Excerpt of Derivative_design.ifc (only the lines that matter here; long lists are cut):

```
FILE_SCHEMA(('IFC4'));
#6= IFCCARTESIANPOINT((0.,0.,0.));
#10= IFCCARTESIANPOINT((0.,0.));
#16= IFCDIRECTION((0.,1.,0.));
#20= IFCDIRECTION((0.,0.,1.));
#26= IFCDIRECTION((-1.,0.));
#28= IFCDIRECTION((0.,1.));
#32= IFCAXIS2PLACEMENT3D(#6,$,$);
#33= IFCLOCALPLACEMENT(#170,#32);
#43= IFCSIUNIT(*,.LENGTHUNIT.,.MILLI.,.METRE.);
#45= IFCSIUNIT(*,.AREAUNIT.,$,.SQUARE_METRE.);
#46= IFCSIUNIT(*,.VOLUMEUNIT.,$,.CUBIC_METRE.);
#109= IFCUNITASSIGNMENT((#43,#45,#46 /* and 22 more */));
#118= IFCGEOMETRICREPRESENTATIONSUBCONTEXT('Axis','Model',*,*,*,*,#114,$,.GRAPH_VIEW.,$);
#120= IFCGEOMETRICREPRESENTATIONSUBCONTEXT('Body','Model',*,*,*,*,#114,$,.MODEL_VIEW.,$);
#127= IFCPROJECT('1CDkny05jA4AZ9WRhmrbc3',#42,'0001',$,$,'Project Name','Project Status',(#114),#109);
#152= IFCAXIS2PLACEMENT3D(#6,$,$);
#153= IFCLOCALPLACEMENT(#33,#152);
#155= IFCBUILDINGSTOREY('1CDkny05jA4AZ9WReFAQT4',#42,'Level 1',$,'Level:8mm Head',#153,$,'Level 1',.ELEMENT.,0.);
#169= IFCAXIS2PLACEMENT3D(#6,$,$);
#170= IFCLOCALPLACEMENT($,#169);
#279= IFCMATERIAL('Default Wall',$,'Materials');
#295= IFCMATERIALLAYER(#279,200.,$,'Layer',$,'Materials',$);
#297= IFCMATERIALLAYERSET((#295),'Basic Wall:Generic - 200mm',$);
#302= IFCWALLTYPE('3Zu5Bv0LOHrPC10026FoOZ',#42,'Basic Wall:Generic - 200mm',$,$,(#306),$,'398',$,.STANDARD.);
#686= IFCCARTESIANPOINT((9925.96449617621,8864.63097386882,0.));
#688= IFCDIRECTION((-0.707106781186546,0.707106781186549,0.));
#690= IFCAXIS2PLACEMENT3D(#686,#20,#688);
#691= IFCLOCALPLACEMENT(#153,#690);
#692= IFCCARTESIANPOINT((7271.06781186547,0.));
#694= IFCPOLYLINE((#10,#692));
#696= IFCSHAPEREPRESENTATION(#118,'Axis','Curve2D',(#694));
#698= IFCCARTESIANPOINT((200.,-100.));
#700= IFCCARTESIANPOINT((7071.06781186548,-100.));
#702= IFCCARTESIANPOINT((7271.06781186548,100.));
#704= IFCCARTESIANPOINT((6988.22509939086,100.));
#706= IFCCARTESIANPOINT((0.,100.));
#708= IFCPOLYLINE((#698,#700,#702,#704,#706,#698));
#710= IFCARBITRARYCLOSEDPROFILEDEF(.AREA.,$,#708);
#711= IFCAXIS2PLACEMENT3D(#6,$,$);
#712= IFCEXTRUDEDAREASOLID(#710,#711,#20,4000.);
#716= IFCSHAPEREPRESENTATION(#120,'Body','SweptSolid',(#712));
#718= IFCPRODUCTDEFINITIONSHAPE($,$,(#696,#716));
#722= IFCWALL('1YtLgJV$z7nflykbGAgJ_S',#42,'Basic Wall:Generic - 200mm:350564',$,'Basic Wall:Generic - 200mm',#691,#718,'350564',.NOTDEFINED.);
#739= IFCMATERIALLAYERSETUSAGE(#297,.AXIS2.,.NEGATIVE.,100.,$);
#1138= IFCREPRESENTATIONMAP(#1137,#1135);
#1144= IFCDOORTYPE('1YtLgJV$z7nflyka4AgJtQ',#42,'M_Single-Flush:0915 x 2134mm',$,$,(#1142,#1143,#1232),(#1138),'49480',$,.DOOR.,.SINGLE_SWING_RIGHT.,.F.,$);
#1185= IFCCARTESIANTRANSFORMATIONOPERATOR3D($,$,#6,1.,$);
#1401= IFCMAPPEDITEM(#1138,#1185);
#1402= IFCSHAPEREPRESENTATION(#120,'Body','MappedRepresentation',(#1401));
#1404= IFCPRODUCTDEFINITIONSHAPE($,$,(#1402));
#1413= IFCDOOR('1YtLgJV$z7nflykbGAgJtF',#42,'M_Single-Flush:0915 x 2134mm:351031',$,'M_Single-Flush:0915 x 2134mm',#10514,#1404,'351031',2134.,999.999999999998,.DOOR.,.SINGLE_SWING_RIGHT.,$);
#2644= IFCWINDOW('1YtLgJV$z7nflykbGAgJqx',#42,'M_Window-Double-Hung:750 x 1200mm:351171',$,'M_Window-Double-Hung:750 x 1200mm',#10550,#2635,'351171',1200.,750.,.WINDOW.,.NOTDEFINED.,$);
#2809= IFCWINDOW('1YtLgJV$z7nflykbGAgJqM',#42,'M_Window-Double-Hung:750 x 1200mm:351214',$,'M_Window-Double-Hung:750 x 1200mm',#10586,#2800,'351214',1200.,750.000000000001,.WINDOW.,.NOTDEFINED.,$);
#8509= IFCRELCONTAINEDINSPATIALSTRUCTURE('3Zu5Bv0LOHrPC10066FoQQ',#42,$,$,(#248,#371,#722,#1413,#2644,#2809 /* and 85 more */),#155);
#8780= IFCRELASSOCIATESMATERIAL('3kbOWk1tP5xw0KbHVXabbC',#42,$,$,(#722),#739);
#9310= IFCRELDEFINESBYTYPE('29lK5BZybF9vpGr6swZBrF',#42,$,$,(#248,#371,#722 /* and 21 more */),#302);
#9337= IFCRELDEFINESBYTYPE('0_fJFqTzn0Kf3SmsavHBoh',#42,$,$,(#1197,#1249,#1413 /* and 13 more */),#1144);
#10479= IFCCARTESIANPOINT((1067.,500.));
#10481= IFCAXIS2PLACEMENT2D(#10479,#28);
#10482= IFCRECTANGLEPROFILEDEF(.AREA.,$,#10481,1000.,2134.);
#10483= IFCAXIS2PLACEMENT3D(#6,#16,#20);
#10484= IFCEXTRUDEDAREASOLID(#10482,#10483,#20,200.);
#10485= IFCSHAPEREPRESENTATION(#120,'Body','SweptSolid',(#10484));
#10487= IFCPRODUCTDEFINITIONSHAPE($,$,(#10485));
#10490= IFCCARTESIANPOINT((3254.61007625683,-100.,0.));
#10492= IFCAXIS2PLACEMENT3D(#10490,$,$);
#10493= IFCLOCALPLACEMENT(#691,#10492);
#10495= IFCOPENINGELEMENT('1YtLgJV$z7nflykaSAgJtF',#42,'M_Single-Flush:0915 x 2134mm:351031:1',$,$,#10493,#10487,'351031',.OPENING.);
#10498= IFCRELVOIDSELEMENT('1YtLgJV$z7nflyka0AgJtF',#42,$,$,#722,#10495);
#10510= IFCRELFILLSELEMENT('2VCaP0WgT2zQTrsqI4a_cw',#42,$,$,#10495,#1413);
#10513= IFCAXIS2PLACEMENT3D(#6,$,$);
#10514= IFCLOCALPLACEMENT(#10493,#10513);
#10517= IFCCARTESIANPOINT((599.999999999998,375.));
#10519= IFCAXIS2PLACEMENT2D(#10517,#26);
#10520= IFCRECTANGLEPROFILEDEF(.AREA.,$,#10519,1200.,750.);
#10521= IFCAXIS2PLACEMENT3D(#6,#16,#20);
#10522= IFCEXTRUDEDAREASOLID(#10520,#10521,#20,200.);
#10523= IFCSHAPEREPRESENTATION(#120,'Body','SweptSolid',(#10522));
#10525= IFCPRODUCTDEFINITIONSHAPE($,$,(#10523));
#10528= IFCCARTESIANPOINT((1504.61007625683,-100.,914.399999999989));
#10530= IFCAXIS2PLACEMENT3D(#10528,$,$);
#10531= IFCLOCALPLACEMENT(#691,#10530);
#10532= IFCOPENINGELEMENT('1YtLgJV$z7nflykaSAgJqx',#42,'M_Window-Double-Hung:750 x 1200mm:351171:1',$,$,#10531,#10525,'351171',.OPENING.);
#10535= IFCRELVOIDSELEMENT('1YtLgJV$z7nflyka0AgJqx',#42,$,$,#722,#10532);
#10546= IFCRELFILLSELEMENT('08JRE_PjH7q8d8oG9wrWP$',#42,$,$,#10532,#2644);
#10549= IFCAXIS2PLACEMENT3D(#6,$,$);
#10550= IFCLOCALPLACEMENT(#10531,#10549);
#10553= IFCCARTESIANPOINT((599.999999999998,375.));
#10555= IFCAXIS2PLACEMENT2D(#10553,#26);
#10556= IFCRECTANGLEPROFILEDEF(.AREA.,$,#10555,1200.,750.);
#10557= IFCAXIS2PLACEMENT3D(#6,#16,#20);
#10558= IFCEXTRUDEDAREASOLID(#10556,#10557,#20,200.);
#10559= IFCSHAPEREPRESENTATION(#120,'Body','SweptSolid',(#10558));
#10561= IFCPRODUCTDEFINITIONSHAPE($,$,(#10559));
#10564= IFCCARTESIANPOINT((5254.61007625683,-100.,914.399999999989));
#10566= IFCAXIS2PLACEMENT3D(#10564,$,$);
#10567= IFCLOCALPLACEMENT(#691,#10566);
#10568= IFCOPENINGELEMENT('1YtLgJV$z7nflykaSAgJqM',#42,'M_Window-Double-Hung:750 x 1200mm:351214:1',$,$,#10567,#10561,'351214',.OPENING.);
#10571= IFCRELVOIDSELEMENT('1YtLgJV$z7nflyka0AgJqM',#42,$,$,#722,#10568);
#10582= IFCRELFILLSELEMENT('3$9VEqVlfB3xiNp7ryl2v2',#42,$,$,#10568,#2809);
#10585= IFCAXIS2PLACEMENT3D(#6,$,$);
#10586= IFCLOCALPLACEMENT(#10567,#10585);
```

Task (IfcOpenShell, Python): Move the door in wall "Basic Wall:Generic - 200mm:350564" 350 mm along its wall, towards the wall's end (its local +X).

```python
import ifcopenshell
import ifcopenshell.api.geometry
import ifcopenshell.util.placement
import ifcopenshell.util.unit

model = ifcopenshell.open("Derivative_design.ifc")
unit_scale = ifcopenshell.util.unit.calculate_unit_scale(model)

door = model.by_guid("1YtLgJV$z7nflykbGAgJtF")
opening = door.FillsVoids[0].RelatingOpeningElement
wall = opening.VoidsElements[0].RelatingBuildingElement

wall_matrix = ifcopenshell.util.placement.get_local_placement(wall.ObjectPlacement)
shift = wall_matrix[:3, 0] * 0.35 / unit_scale
before = ifcopenshell.util.placement.get_local_placement(door.ObjectPlacement)[:3, 3].copy()

# The door is placed relative to its opening, so it follows when the opening moves.
matrix = ifcopenshell.util.placement.get_local_placement(opening.ObjectPlacement)
matrix[:3, 3] += shift
ifcopenshell.api.geometry.edit_object_placement(
    model, product=opening, matrix=matrix, is_si=False, should_transform_children=True
)

after = ifcopenshell.util.placement.get_local_placement(door.ObjectPlacement)[:3, 3]
print("door moved by", (after - before).round(3) + 0.0)

model.write("Derivative_design_updated.ifc")
```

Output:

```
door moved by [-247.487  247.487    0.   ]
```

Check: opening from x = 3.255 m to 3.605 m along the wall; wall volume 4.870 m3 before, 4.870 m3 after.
